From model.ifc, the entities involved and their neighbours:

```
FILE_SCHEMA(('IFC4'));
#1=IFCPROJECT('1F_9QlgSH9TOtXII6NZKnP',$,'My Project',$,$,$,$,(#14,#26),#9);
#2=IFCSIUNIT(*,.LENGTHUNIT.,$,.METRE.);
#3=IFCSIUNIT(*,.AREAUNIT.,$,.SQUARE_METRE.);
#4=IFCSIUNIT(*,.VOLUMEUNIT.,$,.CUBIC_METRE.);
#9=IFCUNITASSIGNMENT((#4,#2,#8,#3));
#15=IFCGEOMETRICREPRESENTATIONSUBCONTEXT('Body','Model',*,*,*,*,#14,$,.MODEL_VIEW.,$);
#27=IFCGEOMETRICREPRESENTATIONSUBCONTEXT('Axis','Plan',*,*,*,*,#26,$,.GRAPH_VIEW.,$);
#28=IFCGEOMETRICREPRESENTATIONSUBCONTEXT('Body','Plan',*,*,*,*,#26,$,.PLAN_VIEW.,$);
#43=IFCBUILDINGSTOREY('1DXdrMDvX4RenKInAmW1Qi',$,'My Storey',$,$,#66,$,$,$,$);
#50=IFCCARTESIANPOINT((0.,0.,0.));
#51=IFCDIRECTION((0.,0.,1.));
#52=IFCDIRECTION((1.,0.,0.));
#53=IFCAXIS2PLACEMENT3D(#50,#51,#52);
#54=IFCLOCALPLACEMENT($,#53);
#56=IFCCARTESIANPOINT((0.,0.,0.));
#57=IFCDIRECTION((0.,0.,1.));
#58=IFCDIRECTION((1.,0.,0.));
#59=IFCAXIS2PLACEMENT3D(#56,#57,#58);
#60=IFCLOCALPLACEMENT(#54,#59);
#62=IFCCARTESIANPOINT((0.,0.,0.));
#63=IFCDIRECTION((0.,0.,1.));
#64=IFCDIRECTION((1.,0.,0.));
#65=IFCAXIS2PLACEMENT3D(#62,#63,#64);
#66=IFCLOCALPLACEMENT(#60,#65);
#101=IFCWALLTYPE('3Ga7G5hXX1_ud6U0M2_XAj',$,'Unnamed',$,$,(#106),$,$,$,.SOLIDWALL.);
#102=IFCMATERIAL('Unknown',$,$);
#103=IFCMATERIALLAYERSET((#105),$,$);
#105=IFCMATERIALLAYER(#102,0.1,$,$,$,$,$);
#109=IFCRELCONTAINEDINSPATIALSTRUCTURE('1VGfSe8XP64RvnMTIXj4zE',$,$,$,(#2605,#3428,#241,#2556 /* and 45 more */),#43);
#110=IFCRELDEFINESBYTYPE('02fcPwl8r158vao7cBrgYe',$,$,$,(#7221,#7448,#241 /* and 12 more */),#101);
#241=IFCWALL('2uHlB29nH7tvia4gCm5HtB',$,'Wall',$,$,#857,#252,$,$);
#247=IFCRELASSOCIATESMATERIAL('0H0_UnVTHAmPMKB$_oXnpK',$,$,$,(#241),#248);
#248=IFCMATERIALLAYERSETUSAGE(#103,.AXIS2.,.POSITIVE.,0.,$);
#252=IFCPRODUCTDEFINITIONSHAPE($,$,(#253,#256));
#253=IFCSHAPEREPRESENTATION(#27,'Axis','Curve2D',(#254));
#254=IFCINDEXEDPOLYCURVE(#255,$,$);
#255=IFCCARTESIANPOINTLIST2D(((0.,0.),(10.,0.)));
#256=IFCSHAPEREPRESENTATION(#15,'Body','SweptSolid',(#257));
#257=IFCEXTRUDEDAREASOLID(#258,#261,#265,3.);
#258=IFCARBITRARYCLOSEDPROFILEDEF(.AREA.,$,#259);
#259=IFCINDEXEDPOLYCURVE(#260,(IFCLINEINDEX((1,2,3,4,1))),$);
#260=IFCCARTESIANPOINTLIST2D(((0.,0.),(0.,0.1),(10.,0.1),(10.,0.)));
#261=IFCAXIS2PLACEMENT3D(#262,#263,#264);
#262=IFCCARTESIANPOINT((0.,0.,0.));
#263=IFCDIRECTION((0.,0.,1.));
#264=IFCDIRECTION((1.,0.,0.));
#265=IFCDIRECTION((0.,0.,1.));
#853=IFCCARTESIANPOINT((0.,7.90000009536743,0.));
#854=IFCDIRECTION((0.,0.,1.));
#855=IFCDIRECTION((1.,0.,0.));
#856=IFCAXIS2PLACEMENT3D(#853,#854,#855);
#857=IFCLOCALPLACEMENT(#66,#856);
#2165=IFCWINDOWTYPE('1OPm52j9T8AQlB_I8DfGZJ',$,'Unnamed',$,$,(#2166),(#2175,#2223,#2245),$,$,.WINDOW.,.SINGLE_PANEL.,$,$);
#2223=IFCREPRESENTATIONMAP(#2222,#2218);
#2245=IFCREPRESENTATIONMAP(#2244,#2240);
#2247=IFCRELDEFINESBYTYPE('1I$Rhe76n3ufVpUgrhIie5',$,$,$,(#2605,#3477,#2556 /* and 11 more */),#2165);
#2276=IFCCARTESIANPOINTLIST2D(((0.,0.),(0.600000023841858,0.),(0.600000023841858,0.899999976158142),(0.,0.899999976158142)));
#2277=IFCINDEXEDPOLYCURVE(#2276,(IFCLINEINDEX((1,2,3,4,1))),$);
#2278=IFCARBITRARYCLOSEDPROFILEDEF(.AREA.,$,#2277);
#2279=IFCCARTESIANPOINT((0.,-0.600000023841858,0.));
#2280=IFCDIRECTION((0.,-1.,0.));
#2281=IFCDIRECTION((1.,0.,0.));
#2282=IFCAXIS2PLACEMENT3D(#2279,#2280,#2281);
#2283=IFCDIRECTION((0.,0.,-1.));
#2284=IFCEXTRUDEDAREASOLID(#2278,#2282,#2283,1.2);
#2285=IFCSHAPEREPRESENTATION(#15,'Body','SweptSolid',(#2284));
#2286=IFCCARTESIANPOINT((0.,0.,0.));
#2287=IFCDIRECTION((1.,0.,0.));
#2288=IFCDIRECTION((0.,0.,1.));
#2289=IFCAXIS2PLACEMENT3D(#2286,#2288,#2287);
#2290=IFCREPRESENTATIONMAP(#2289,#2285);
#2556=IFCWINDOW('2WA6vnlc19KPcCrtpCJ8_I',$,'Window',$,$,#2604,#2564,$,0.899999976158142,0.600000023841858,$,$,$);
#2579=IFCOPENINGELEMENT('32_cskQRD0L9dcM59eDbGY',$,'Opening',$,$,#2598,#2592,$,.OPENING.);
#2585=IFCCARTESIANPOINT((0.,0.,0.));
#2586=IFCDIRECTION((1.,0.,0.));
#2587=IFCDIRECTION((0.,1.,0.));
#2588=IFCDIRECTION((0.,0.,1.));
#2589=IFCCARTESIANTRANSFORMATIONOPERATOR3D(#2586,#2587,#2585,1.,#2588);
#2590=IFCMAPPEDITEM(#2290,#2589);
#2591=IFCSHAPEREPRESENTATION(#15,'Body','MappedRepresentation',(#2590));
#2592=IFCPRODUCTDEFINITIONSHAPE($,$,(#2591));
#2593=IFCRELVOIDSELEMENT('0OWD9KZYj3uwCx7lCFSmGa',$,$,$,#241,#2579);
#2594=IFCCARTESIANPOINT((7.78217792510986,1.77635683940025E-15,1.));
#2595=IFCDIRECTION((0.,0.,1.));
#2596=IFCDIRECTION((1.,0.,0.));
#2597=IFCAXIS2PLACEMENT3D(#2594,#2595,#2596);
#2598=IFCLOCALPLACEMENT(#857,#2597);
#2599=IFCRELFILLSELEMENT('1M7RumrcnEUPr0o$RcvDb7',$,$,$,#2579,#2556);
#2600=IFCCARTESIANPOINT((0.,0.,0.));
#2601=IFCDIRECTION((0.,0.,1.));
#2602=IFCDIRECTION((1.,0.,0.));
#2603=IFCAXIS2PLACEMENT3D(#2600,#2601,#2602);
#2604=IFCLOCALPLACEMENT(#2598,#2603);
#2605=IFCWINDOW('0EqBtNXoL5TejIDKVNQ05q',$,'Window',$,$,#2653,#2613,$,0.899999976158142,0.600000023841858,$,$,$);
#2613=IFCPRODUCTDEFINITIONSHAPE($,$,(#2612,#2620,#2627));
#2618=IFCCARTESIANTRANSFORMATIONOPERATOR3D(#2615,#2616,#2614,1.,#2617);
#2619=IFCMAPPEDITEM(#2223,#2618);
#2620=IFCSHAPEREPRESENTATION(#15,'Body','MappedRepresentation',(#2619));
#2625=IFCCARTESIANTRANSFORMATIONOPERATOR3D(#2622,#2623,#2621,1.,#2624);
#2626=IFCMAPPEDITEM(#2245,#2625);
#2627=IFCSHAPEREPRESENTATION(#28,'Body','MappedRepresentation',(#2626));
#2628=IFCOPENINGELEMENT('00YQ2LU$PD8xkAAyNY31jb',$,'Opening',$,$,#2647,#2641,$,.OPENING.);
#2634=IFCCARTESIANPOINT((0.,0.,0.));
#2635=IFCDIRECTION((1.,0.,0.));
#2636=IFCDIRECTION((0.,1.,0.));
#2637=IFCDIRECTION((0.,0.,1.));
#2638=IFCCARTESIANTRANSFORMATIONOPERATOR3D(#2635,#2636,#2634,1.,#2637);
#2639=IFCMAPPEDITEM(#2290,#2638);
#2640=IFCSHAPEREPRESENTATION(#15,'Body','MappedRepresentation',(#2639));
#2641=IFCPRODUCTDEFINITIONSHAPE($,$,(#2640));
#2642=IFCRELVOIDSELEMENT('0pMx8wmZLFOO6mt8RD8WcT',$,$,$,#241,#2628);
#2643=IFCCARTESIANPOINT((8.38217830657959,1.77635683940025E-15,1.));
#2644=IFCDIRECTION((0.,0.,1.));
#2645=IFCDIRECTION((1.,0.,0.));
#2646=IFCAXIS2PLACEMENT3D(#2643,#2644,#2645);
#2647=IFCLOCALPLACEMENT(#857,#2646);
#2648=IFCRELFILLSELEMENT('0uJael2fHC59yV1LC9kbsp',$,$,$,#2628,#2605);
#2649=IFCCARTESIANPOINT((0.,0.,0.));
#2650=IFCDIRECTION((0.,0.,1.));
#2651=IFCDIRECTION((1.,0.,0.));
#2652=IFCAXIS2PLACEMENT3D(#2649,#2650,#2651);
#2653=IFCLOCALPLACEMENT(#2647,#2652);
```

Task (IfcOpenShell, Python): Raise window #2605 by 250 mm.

```python
import numpy as np
import ifcopenshell
import ifcopenshell.api.geometry
import ifcopenshell.util.placement
import ifcopenshell.util.unit

model = ifcopenshell.open("model.ifc")
unit_scale = ifcopenshell.util.unit.calculate_unit_scale(model)

window = model.by_guid("0EqBtNXoL5TejIDKVNQ05q")
opening = window.FillsVoids[0].RelatingOpeningElement
dz = 0.25 / unit_scale

shift = np.array([0.0, 0.0, dz])
# The window is placed relative to its opening, so it follows when the opening moves.
matrix = ifcopenshell.util.placement.get_local_placement(opening.ObjectPlacement)
matrix[:3, 3] += shift
ifcopenshell.api.geometry.edit_object_placement(
    model, product=opening, matrix=matrix, is_si=False, should_transform_children=True
)

print(f"moved by {dz * unit_scale:+.3f} m")

model.write("model-out.ifc")
```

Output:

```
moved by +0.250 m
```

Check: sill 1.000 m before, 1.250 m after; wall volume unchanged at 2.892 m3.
